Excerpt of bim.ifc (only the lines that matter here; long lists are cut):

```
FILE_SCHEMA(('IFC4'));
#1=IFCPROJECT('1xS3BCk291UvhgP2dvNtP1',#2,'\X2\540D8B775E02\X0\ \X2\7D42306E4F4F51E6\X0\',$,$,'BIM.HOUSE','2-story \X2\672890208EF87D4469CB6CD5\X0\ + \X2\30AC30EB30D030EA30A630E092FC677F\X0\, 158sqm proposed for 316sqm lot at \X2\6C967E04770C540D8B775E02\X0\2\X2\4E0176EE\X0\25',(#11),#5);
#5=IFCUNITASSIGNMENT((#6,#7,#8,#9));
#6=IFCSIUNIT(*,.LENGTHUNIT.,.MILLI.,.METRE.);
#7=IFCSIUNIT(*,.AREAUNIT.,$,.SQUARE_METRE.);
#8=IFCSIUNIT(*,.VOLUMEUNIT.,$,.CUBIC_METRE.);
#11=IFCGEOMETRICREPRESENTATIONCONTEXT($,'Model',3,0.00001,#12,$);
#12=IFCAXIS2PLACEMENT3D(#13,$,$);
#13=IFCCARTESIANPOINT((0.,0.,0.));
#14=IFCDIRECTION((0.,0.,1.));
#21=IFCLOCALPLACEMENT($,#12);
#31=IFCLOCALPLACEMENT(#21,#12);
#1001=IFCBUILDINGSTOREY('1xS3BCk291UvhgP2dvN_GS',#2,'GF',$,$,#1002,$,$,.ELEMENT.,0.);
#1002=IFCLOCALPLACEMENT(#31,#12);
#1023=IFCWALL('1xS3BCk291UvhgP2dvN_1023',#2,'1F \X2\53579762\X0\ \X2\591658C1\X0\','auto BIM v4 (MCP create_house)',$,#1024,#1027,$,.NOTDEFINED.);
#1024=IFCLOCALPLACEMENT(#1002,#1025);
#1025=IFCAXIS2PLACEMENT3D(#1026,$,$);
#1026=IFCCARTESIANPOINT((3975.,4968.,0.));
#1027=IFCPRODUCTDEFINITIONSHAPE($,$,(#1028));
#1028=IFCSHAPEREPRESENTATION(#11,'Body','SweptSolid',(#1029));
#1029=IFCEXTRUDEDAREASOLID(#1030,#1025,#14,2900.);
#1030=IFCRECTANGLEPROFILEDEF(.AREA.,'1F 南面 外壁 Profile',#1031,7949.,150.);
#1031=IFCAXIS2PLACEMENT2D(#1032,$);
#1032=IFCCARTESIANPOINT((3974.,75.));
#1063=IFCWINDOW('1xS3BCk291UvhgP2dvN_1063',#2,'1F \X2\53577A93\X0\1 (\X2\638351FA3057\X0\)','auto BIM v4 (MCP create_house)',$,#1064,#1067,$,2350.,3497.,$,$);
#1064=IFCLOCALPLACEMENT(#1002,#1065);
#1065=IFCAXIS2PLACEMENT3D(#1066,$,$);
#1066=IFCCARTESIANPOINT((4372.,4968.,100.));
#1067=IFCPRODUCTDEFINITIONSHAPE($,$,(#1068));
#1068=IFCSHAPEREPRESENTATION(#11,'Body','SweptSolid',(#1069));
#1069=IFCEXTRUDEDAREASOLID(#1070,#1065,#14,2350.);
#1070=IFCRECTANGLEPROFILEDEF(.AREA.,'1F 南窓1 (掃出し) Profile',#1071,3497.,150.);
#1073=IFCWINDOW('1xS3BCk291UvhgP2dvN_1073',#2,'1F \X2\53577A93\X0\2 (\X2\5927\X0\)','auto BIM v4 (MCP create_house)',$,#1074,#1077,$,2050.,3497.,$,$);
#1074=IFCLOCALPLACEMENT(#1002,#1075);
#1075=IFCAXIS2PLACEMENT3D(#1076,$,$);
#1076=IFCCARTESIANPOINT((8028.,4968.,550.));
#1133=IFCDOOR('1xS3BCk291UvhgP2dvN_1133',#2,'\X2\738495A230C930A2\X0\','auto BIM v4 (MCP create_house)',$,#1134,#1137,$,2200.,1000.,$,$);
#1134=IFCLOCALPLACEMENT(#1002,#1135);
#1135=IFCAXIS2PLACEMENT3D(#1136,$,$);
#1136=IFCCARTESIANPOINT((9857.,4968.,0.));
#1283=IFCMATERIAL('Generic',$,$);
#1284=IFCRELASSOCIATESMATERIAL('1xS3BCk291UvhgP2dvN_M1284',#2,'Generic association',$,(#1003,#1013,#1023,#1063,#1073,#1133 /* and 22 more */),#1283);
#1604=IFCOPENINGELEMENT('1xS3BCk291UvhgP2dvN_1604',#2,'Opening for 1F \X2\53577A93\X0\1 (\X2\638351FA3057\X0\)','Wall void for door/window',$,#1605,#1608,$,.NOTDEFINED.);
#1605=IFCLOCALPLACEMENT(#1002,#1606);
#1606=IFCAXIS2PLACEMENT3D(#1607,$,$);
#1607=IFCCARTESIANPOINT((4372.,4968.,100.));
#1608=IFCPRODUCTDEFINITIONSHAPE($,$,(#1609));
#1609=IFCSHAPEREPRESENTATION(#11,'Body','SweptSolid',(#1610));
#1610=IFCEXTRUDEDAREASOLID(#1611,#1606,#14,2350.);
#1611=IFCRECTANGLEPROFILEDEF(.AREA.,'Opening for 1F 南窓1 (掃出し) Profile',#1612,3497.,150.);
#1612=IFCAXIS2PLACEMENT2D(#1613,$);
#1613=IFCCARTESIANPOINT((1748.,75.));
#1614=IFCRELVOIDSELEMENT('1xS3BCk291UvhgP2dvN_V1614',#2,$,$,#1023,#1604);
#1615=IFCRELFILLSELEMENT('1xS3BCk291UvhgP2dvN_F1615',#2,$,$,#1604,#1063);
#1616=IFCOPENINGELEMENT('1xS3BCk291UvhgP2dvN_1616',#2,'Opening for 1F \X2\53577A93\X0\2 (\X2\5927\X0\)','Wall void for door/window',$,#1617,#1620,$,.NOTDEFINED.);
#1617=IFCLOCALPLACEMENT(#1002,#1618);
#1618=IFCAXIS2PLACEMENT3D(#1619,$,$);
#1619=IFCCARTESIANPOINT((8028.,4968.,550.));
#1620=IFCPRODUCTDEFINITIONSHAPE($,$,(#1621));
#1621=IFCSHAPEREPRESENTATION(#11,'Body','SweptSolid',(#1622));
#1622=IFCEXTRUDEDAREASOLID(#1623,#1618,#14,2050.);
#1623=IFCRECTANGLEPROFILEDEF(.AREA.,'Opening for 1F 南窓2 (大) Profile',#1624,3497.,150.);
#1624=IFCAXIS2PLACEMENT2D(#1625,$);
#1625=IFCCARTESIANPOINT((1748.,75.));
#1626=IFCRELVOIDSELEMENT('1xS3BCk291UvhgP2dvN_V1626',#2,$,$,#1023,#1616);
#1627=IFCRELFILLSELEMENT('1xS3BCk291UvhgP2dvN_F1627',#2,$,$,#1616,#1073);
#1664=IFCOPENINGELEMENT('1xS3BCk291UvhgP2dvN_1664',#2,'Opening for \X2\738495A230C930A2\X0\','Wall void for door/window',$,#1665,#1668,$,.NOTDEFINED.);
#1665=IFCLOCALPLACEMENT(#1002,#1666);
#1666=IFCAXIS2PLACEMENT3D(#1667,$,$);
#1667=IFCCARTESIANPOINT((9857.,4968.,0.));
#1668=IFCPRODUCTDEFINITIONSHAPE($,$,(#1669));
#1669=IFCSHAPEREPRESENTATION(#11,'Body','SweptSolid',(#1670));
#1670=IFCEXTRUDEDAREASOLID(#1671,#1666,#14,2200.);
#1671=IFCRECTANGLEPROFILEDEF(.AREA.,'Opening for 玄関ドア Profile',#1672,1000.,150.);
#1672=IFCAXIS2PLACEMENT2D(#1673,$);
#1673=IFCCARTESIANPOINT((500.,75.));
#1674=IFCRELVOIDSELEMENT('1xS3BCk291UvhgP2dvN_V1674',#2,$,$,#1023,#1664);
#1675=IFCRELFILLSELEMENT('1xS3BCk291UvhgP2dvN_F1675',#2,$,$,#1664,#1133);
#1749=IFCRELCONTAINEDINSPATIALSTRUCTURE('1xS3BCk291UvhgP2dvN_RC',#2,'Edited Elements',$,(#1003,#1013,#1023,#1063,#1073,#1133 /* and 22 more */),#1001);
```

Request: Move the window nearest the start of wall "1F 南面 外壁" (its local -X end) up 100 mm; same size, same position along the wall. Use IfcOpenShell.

```python
import numpy as np
import ifcopenshell
import ifcopenshell.api.geometry
import ifcopenshell.util.placement
import ifcopenshell.util.unit

model = ifcopenshell.open("bim.ifc")
unit_scale = ifcopenshell.util.unit.calculate_unit_scale(model)

window = model.by_guid("1xS3BCk291UvhgP2dvN_1063")
opening = window.FillsVoids[0].RelatingOpeningElement
dz = 100.0

shift = np.array([0.0, 0.0, dz])
# The window is not placed relative to its opening, so move both.
for product in (opening, window):
    matrix = ifcopenshell.util.placement.get_local_placement(product.ObjectPlacement)
    matrix[:3, 3] += shift
    ifcopenshell.api.geometry.edit_object_placement(model, product=product, matrix=matrix, is_si=False)

print(f"moved by {dz * unit_scale:+.3f} m")

model.write("bim-out.ifc")
```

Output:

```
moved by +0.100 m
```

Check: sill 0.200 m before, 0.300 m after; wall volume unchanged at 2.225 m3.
